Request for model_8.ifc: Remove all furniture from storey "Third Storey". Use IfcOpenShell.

First a look at what the model holds.

```python
import ifcopenshell
import ifcopenshell.util.element

model = ifcopenshell.open("model_8.ifc")
print(model.schema)
storey = next(s for s in model.by_type("IfcBuildingStorey") if s.Name == "Third Storey")
furniture = [e for e in ifcopenshell.util.element.get_decomposition(storey) if e.is_a("IfcFurnishingElement")]
seen = {}
for e in furniture:
    element_type = ifcopenshell.util.element.get_type(e)
    name = element_type.Name if element_type not in (None, e) else None
    seen[name] = seen.get(name, 0) + 1
for name, count in sorted(seen.items(), key=str):
    print(count, "x", name)
```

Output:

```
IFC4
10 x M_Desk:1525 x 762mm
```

```python
import ifcopenshell
import ifcopenshell.api.root
import ifcopenshell.util.element

model = ifcopenshell.open("model_8.ifc")

storey = next(s for s in model.by_type("IfcBuildingStorey") if s.Name == "Third Storey")
furniture = [e for e in ifcopenshell.util.element.get_decomposition(storey) if e.is_a("IfcFurnishingElement")]

for e in furniture:
    ifcopenshell.api.root.remove_product(model, product=e)
print(len(furniture), "removed")

model.write("model_8_v2.ifc")
```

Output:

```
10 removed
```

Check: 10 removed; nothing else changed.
